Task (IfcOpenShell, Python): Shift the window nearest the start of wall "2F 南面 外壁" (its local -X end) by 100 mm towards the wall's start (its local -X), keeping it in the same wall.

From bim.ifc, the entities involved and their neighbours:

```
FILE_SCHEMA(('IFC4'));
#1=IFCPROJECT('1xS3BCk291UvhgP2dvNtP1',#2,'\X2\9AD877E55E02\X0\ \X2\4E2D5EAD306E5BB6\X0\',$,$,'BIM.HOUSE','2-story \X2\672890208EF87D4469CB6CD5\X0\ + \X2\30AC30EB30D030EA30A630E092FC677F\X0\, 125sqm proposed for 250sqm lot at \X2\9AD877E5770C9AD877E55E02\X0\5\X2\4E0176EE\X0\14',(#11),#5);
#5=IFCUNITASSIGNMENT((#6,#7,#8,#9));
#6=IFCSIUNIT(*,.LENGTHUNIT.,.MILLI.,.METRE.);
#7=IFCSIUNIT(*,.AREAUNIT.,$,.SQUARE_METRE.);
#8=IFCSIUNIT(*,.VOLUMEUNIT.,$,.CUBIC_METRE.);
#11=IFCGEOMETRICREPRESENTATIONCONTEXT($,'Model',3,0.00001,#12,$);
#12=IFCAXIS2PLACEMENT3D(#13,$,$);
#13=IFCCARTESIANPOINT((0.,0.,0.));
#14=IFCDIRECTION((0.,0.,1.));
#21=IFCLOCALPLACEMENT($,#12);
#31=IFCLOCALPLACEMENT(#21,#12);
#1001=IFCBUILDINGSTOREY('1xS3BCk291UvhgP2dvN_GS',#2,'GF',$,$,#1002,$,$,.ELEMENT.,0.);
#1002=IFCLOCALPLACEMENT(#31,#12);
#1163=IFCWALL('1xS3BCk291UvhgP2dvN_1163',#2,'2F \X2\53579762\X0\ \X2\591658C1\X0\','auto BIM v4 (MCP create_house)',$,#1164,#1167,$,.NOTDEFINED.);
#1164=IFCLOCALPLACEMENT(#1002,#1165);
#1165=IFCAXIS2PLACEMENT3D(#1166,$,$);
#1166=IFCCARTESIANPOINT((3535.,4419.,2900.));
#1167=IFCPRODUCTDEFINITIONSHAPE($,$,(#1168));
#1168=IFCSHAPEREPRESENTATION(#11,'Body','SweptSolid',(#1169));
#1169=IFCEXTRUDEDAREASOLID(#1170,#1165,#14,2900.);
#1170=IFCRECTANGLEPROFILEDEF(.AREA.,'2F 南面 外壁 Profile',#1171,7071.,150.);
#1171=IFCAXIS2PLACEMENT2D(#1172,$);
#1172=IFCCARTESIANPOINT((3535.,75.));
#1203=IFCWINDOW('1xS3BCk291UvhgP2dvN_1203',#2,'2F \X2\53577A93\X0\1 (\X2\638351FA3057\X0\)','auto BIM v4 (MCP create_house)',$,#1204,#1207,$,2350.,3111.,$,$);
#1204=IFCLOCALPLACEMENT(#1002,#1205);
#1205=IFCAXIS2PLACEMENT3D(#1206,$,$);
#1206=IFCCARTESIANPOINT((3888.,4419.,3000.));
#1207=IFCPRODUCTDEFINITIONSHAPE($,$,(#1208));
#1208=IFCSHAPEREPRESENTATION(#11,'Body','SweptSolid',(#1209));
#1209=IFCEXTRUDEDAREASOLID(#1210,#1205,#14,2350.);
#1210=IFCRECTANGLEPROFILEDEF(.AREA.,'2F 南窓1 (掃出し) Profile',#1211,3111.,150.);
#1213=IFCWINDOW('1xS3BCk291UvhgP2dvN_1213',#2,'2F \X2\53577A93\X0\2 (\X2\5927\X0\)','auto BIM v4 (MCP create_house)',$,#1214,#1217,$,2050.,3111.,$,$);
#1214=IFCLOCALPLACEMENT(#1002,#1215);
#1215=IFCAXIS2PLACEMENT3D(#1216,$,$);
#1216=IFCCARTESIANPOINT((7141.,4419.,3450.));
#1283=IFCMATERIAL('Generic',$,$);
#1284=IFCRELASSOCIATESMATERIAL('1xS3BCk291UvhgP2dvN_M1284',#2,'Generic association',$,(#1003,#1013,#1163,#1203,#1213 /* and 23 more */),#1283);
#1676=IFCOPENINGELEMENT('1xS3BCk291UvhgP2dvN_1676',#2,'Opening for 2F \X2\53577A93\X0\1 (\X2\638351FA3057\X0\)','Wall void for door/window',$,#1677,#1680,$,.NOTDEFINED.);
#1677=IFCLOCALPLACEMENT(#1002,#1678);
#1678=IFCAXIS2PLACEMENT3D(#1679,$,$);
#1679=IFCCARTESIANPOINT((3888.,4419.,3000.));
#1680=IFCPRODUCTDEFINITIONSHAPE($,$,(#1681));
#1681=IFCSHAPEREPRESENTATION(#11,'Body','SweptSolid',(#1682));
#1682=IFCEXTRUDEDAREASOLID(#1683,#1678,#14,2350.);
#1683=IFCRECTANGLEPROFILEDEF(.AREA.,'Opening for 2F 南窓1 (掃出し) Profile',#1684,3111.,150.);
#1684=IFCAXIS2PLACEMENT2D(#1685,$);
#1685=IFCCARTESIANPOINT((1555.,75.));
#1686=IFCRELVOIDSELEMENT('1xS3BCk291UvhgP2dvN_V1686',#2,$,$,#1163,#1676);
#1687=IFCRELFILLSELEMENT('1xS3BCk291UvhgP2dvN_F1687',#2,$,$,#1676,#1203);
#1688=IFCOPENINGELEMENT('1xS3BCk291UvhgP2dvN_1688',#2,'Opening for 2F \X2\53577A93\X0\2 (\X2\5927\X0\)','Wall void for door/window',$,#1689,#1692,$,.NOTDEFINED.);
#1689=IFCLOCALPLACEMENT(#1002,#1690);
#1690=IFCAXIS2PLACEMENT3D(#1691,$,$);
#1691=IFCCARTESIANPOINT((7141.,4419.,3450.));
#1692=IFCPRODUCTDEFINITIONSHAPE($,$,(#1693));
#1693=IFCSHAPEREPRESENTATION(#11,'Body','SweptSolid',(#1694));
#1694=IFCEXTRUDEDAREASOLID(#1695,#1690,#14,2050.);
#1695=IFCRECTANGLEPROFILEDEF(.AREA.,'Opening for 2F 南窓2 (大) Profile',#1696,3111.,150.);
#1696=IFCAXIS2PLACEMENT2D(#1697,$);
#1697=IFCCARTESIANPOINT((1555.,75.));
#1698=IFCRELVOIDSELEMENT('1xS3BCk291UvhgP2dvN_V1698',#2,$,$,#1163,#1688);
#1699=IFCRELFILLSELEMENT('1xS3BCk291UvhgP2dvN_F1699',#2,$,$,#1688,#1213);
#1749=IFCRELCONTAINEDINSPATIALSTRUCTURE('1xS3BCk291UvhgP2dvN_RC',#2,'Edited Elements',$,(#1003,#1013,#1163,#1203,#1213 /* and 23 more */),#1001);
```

```python
import ifcopenshell
import ifcopenshell.api.geometry
import ifcopenshell.util.placement
import ifcopenshell.util.unit

model = ifcopenshell.open("bim.ifc")
unit_scale = ifcopenshell.util.unit.calculate_unit_scale(model)

window = model.by_guid("1xS3BCk291UvhgP2dvN_1203")
opening = window.FillsVoids[0].RelatingOpeningElement
wall = opening.VoidsElements[0].RelatingBuildingElement

wall_matrix = ifcopenshell.util.placement.get_local_placement(wall.ObjectPlacement)
shift = wall_matrix[:3, 0] * -0.1 / unit_scale
before = ifcopenshell.util.placement.get_local_placement(window.ObjectPlacement)[:3, 3].copy()

# The window is not placed relative to its opening, so move both.
for product in (opening, window):
    matrix = ifcopenshell.util.placement.get_local_placement(product.ObjectPlacement)
    matrix[:3, 3] += shift
    ifcopenshell.api.geometry.edit_object_placement(model, product=product, matrix=matrix, is_si=False)

after = ifcopenshell.util.placement.get_local_placement(window.ObjectPlacement)[:3, 3]
print("window moved by", (after - before).round(3) + 0.0)

model.write("bim_updated.ifc")
```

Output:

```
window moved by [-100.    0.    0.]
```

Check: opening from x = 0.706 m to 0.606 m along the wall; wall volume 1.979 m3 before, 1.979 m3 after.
